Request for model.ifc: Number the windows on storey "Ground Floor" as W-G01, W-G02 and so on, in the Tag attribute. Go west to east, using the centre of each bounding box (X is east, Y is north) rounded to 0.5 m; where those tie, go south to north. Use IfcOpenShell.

First a look at what the model holds.

```python
import ifcopenshell
import ifcopenshell.util.element
import ifcopenshell.util.placement

model = ifcopenshell.open("model.ifc")
print(model.schema)
storey = next(s for s in model.by_type("IfcBuildingStorey") if s.Name == "Ground Floor")
windows = [e for e in ifcopenshell.util.element.get_decomposition(storey) if e.is_a("IfcWindow")]
for e in sorted(windows, key=lambda e: e.id()):
    origin = ifcopenshell.util.placement.get_local_placement(e.ObjectPlacement)[:3, 3]
    print(e.id(), e.Tag, e.Name, origin.round(2) + 0.0, sep=" | ")
```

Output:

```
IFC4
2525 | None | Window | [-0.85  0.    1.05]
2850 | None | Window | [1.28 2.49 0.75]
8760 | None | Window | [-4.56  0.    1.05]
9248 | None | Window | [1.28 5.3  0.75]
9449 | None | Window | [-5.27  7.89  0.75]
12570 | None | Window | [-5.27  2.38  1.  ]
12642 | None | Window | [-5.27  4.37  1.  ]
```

```python
import ifcopenshell
import ifcopenshell.geom
import ifcopenshell.util.element
import ifcopenshell.util.shape

model = ifcopenshell.open("model.ifc")
settings = ifcopenshell.geom.settings()
settings.set("use-world-coords", True)


def centre(element):
    shape = ifcopenshell.geom.create_shape(settings, element)
    return ifcopenshell.util.shape.get_bbox_centroid(shape.geometry)


storey = next(s for s in model.by_type("IfcBuildingStorey") if s.Name == "Ground Floor")
windows = [e for e in ifcopenshell.util.element.get_decomposition(storey) if e.is_a("IfcWindow")]

# Insertion points can sit at a corner or the storey origin, so sort by the geometry (in metres).
centres = {e: centre(e) for e in windows}
windows.sort(key=lambda e: (round(centres[e][0] / 0.5), centres[e][1]))

for i, e in enumerate(windows, start=1):
    number = f"W-G{i:02d}"
    e.Tag = number
    print(e.id(), number)

model.write("model_updated.ifc")
```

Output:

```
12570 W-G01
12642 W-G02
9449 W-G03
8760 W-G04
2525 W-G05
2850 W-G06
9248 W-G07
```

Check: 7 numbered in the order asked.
